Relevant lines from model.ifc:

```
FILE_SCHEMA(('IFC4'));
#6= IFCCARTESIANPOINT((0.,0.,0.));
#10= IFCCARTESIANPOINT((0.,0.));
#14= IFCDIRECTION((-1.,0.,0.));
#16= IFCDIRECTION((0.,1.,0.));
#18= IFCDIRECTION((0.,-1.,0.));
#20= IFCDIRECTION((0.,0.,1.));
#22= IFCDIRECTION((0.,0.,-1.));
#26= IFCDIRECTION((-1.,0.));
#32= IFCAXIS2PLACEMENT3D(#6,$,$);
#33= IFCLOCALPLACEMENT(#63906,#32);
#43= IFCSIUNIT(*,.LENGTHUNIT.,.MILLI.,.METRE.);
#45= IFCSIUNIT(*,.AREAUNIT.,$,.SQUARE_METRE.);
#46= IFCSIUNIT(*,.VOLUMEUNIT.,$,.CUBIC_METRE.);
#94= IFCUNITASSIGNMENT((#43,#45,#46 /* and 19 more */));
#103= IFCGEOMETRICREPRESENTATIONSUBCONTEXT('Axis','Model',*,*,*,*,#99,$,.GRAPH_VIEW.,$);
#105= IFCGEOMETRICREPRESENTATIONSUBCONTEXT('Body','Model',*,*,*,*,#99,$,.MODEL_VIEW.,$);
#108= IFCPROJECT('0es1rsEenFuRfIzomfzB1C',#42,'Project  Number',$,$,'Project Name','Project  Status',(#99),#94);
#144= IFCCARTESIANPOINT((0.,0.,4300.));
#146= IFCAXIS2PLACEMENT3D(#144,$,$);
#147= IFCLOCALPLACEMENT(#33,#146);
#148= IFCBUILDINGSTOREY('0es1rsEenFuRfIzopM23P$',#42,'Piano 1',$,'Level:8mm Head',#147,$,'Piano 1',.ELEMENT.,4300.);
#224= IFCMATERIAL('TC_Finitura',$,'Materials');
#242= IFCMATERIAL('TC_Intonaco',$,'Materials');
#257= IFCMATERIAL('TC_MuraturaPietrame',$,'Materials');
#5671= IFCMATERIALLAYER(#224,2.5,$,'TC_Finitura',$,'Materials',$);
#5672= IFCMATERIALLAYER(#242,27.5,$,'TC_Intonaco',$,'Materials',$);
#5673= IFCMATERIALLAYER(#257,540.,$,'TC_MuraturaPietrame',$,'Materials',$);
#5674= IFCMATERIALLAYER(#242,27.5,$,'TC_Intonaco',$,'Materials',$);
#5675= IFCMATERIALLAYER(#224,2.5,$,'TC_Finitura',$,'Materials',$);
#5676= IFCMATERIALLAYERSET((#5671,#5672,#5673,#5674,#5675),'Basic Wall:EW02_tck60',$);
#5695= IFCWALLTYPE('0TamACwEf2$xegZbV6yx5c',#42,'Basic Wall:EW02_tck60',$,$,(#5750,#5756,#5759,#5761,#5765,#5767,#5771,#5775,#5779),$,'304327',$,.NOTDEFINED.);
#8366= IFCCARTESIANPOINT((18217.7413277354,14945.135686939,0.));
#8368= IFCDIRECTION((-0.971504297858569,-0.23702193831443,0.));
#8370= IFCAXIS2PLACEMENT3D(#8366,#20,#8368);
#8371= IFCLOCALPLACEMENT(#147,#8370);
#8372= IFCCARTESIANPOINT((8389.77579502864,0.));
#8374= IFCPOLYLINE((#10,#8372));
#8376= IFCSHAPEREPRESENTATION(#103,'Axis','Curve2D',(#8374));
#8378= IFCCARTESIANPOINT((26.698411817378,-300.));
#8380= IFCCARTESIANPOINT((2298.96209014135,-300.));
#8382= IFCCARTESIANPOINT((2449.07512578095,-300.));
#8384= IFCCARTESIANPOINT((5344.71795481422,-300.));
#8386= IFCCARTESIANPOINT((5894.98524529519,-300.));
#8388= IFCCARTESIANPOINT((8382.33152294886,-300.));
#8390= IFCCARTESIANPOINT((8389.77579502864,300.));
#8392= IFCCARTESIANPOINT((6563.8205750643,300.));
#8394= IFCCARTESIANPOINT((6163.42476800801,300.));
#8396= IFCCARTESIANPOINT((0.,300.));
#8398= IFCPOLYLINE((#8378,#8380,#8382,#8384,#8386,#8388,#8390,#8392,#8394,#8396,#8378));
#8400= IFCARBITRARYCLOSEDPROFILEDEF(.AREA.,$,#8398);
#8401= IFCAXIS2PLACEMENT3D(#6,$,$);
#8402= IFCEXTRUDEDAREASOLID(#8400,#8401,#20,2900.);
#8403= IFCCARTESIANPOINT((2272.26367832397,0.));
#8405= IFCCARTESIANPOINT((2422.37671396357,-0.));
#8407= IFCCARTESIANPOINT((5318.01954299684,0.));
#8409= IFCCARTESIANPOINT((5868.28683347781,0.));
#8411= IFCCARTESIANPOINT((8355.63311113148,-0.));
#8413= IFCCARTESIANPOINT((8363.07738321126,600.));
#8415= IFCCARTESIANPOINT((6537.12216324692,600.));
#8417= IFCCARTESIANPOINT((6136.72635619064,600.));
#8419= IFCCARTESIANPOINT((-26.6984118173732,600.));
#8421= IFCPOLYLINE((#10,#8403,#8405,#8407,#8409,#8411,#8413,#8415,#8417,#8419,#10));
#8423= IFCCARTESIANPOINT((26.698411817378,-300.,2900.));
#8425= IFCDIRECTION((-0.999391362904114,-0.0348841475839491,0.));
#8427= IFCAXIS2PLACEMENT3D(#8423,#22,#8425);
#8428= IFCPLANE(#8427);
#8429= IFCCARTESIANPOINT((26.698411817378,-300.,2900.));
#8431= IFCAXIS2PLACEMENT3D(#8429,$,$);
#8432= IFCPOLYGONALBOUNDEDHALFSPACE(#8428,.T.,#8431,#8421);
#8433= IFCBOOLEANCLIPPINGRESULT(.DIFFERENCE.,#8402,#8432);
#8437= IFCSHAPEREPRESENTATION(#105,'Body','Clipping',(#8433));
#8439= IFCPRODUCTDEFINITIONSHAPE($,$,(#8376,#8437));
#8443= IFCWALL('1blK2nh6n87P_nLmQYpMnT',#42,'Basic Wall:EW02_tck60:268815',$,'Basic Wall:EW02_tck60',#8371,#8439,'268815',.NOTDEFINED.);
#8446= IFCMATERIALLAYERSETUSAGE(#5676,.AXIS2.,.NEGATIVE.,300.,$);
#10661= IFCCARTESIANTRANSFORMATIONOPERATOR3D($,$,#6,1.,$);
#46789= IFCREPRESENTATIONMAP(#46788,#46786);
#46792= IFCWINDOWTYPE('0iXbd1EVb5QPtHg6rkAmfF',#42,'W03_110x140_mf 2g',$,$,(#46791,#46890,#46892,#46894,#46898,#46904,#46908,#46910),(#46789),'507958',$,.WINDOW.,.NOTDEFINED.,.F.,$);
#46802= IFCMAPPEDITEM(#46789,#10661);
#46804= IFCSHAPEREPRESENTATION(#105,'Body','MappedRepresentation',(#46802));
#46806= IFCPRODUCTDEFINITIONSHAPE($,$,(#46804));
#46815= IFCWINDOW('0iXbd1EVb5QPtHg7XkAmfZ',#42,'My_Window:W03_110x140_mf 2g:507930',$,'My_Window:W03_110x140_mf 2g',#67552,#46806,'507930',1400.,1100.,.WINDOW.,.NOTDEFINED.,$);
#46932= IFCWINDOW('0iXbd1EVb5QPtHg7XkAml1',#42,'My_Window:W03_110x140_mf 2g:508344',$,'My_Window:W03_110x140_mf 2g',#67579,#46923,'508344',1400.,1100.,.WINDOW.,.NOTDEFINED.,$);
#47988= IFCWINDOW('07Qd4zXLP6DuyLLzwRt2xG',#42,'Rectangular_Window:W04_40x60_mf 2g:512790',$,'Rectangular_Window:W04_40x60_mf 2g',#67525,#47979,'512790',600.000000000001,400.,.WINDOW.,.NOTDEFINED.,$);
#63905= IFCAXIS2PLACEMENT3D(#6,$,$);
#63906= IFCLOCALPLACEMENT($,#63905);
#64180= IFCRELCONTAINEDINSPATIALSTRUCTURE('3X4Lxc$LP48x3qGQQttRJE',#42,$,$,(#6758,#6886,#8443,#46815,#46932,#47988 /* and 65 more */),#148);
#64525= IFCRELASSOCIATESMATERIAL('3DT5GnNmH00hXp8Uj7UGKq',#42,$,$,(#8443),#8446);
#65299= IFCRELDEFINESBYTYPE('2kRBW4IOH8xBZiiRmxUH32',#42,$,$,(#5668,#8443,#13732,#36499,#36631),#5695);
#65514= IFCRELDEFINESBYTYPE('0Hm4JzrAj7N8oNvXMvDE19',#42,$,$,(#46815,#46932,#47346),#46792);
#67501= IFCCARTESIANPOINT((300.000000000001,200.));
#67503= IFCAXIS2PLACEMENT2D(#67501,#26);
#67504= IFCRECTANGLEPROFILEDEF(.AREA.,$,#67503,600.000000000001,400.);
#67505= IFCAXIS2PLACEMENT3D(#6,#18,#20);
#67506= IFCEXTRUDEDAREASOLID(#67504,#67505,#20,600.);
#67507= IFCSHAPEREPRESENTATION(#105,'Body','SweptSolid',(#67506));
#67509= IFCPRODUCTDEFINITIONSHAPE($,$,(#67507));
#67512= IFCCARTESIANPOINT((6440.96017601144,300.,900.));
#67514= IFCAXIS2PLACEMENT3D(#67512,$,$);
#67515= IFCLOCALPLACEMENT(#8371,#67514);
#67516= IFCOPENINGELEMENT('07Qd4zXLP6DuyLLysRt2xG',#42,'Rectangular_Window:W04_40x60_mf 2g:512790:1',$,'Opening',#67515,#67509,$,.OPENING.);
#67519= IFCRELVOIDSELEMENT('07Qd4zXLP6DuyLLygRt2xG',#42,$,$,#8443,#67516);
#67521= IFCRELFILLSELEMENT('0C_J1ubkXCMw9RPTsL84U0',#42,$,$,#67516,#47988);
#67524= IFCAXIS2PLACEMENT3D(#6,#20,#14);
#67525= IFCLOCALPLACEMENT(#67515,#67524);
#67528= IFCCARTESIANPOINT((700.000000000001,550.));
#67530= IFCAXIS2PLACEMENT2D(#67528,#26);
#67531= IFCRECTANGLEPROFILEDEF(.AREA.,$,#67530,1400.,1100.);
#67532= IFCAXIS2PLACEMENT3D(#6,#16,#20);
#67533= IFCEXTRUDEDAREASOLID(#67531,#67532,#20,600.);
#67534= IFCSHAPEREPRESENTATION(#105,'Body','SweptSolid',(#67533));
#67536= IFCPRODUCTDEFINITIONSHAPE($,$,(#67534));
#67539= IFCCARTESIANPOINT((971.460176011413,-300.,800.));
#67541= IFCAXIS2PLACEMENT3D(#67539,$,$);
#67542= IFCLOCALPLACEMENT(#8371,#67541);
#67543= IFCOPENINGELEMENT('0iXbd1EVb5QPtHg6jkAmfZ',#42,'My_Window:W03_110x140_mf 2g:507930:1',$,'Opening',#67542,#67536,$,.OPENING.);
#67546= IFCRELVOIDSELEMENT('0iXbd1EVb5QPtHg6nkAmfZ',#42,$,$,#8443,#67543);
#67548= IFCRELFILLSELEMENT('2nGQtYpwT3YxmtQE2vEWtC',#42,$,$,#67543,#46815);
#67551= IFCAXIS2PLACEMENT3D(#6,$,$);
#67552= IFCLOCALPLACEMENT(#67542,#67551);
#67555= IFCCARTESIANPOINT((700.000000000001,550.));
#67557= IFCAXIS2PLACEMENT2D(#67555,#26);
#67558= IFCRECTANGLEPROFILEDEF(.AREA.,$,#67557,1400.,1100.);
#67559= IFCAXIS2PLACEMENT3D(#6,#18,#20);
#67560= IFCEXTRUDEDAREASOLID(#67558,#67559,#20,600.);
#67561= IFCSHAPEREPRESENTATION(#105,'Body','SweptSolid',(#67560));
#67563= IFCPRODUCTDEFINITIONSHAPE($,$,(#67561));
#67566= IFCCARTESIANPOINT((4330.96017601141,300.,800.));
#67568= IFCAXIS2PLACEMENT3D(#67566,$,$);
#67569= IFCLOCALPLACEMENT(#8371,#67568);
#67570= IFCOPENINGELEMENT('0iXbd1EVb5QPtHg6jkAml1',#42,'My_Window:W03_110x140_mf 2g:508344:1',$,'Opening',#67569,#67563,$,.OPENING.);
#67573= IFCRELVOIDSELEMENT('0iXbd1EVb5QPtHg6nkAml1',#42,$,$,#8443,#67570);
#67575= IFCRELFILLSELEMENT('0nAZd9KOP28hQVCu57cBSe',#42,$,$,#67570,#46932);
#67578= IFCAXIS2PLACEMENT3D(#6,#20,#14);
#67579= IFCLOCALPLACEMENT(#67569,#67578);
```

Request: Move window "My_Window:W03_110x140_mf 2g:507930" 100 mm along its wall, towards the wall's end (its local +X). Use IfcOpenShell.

```python
import ifcopenshell
import ifcopenshell.api.geometry
import ifcopenshell.util.placement

model = ifcopenshell.open("model.ifc")

window = model.by_guid("0iXbd1EVb5QPtHg7XkAmfZ")
opening = window.FillsVoids[0].RelatingOpeningElement
wall = opening.VoidsElements[0].RelatingBuildingElement

wall_matrix = ifcopenshell.util.placement.get_local_placement(wall.ObjectPlacement)
shift = wall_matrix[:3, 0] * 100.0
before = ifcopenshell.util.placement.get_local_placement(window.ObjectPlacement)[:3, 3].copy()

# The window is placed relative to its opening, so it follows when the opening moves.
matrix = ifcopenshell.util.placement.get_local_placement(opening.ObjectPlacement)
matrix[:3, 3] += shift
ifcopenshell.api.geometry.edit_object_placement(
    model, product=opening, matrix=matrix, is_si=False, should_transform_children=True
)

after = ifcopenshell.util.placement.get_local_placement(window.ObjectPlacement)[:3, 3]
print("window moved by", (after - before).round(3) + 0.0)

model.write("model_v2.ifc")
```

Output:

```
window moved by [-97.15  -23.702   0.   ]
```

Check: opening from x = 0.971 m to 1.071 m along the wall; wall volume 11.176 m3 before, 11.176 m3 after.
